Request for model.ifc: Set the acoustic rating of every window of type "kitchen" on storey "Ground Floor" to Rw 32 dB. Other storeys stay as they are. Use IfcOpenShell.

First a look at what the model holds.

```python
import ifcopenshell
import ifcopenshell.util.element

model = ifcopenshell.open("model.ifc")
print(model.schema)
storey = next(s for s in model.by_type("IfcBuildingStorey") if s.Name == "Ground Floor")
windows = [e for e in ifcopenshell.util.element.get_decomposition(storey) if e.is_a("IfcWindow")]
seen = {}
for e in windows:
    element_type = ifcopenshell.util.element.get_type(e)
    key = (element_type.Name if element_type != e and element_type else None, ifcopenshell.util.element.get_pset(e, "Pset_WindowCommon", "AcousticRating"))
    seen[key] = seen.get(key, 0) + 1
for (name, value), count in sorted(seen.items(), key=str):
    print(count, "x", name, "|", value)
```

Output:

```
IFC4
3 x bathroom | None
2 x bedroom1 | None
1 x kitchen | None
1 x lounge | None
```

```python
import ifcopenshell
import ifcopenshell.api.pset
import ifcopenshell.util.element

model = ifcopenshell.open("model.ifc")

storey = next(s for s in model.by_type("IfcBuildingStorey") if s.Name == "Ground Floor")
windows = [e for e in ifcopenshell.util.element.get_decomposition(storey) if e.is_a("IfcWindow")]

count = 0
for e in windows:
    element_type = ifcopenshell.util.element.get_type(e)
    if element_type in (None, e) or element_type.Name != "kitchen":
        continue
    # add_pset returns the element's existing set when there is one.
    pset = ifcopenshell.api.pset.add_pset(model, product=e, name="Pset_WindowCommon")
    ifcopenshell.api.pset.edit_pset(model, pset=pset, properties={"AcousticRating": "Rw 32 dB"})
    count += 1

print(count, "windows updated")

model.write("model_v2.ifc")
```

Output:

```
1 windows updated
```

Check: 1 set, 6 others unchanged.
